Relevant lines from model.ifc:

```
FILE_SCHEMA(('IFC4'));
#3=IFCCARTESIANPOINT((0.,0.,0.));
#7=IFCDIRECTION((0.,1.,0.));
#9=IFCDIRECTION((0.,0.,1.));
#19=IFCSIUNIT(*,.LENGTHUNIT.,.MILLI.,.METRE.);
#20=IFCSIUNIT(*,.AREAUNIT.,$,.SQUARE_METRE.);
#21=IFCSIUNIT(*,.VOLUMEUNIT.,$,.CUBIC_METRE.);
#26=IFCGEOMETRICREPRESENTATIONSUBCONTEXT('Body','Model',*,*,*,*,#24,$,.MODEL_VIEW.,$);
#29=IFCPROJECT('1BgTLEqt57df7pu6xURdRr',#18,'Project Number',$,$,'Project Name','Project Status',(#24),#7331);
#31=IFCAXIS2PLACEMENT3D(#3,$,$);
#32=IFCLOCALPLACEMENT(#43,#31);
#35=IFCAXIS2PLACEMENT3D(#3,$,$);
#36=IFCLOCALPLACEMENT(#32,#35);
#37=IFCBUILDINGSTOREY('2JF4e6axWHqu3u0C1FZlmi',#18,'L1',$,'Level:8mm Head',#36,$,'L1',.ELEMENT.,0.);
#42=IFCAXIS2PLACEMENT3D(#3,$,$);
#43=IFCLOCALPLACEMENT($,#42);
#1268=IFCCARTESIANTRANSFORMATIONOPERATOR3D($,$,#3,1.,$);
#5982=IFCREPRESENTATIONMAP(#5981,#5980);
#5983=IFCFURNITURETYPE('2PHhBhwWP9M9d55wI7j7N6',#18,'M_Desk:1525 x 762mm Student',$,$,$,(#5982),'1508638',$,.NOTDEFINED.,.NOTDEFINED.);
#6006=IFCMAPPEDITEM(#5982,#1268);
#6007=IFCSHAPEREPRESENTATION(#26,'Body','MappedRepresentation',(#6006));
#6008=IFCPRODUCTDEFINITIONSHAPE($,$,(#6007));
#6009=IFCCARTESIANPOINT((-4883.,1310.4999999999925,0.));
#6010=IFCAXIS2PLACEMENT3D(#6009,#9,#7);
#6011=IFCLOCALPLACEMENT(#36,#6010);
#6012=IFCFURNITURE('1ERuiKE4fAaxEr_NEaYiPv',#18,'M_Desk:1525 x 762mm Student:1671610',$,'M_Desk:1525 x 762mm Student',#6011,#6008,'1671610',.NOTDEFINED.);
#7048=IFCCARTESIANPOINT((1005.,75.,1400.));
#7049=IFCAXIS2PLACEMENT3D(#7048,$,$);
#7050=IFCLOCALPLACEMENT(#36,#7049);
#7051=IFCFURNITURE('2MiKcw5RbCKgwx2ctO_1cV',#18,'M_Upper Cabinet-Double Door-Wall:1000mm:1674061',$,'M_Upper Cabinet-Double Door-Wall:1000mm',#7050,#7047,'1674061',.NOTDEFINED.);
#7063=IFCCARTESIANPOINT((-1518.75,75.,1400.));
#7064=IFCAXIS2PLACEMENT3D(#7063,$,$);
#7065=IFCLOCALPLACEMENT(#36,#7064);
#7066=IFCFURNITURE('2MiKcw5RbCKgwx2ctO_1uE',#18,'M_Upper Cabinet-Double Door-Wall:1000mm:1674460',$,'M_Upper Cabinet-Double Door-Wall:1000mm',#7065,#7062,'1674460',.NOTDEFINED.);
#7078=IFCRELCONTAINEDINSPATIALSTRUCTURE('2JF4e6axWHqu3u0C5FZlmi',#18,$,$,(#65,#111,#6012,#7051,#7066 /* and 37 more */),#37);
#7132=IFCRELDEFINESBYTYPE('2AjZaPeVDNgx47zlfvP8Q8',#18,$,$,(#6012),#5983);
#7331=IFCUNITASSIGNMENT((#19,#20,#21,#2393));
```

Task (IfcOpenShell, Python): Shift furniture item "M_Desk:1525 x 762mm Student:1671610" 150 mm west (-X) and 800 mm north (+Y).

```python
import ifcopenshell
import ifcopenshell.api.geometry
import ifcopenshell.util.placement
import ifcopenshell.util.unit

model = ifcopenshell.open("model.ifc")
unit_scale = ifcopenshell.util.unit.calculate_unit_scale(model)

item = model.by_guid("1ERuiKE4fAaxEr_NEaYiPv")
matrix = ifcopenshell.util.placement.get_local_placement(item.ObjectPlacement)
matrix[0, 3] -= 0.15 / unit_scale
matrix[1, 3] += 0.8 / unit_scale
ifcopenshell.api.geometry.edit_object_placement(model, product=item, matrix=matrix, is_si=False)

print(ifcopenshell.util.placement.get_local_placement(item.ObjectPlacement).round(3) + 0.0)

model.write("model-out.ifc")
```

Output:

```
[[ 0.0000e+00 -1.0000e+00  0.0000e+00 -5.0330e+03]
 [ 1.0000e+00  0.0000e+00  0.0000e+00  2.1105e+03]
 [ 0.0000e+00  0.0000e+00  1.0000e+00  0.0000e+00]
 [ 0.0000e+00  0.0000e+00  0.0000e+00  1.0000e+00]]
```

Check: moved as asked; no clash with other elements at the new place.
